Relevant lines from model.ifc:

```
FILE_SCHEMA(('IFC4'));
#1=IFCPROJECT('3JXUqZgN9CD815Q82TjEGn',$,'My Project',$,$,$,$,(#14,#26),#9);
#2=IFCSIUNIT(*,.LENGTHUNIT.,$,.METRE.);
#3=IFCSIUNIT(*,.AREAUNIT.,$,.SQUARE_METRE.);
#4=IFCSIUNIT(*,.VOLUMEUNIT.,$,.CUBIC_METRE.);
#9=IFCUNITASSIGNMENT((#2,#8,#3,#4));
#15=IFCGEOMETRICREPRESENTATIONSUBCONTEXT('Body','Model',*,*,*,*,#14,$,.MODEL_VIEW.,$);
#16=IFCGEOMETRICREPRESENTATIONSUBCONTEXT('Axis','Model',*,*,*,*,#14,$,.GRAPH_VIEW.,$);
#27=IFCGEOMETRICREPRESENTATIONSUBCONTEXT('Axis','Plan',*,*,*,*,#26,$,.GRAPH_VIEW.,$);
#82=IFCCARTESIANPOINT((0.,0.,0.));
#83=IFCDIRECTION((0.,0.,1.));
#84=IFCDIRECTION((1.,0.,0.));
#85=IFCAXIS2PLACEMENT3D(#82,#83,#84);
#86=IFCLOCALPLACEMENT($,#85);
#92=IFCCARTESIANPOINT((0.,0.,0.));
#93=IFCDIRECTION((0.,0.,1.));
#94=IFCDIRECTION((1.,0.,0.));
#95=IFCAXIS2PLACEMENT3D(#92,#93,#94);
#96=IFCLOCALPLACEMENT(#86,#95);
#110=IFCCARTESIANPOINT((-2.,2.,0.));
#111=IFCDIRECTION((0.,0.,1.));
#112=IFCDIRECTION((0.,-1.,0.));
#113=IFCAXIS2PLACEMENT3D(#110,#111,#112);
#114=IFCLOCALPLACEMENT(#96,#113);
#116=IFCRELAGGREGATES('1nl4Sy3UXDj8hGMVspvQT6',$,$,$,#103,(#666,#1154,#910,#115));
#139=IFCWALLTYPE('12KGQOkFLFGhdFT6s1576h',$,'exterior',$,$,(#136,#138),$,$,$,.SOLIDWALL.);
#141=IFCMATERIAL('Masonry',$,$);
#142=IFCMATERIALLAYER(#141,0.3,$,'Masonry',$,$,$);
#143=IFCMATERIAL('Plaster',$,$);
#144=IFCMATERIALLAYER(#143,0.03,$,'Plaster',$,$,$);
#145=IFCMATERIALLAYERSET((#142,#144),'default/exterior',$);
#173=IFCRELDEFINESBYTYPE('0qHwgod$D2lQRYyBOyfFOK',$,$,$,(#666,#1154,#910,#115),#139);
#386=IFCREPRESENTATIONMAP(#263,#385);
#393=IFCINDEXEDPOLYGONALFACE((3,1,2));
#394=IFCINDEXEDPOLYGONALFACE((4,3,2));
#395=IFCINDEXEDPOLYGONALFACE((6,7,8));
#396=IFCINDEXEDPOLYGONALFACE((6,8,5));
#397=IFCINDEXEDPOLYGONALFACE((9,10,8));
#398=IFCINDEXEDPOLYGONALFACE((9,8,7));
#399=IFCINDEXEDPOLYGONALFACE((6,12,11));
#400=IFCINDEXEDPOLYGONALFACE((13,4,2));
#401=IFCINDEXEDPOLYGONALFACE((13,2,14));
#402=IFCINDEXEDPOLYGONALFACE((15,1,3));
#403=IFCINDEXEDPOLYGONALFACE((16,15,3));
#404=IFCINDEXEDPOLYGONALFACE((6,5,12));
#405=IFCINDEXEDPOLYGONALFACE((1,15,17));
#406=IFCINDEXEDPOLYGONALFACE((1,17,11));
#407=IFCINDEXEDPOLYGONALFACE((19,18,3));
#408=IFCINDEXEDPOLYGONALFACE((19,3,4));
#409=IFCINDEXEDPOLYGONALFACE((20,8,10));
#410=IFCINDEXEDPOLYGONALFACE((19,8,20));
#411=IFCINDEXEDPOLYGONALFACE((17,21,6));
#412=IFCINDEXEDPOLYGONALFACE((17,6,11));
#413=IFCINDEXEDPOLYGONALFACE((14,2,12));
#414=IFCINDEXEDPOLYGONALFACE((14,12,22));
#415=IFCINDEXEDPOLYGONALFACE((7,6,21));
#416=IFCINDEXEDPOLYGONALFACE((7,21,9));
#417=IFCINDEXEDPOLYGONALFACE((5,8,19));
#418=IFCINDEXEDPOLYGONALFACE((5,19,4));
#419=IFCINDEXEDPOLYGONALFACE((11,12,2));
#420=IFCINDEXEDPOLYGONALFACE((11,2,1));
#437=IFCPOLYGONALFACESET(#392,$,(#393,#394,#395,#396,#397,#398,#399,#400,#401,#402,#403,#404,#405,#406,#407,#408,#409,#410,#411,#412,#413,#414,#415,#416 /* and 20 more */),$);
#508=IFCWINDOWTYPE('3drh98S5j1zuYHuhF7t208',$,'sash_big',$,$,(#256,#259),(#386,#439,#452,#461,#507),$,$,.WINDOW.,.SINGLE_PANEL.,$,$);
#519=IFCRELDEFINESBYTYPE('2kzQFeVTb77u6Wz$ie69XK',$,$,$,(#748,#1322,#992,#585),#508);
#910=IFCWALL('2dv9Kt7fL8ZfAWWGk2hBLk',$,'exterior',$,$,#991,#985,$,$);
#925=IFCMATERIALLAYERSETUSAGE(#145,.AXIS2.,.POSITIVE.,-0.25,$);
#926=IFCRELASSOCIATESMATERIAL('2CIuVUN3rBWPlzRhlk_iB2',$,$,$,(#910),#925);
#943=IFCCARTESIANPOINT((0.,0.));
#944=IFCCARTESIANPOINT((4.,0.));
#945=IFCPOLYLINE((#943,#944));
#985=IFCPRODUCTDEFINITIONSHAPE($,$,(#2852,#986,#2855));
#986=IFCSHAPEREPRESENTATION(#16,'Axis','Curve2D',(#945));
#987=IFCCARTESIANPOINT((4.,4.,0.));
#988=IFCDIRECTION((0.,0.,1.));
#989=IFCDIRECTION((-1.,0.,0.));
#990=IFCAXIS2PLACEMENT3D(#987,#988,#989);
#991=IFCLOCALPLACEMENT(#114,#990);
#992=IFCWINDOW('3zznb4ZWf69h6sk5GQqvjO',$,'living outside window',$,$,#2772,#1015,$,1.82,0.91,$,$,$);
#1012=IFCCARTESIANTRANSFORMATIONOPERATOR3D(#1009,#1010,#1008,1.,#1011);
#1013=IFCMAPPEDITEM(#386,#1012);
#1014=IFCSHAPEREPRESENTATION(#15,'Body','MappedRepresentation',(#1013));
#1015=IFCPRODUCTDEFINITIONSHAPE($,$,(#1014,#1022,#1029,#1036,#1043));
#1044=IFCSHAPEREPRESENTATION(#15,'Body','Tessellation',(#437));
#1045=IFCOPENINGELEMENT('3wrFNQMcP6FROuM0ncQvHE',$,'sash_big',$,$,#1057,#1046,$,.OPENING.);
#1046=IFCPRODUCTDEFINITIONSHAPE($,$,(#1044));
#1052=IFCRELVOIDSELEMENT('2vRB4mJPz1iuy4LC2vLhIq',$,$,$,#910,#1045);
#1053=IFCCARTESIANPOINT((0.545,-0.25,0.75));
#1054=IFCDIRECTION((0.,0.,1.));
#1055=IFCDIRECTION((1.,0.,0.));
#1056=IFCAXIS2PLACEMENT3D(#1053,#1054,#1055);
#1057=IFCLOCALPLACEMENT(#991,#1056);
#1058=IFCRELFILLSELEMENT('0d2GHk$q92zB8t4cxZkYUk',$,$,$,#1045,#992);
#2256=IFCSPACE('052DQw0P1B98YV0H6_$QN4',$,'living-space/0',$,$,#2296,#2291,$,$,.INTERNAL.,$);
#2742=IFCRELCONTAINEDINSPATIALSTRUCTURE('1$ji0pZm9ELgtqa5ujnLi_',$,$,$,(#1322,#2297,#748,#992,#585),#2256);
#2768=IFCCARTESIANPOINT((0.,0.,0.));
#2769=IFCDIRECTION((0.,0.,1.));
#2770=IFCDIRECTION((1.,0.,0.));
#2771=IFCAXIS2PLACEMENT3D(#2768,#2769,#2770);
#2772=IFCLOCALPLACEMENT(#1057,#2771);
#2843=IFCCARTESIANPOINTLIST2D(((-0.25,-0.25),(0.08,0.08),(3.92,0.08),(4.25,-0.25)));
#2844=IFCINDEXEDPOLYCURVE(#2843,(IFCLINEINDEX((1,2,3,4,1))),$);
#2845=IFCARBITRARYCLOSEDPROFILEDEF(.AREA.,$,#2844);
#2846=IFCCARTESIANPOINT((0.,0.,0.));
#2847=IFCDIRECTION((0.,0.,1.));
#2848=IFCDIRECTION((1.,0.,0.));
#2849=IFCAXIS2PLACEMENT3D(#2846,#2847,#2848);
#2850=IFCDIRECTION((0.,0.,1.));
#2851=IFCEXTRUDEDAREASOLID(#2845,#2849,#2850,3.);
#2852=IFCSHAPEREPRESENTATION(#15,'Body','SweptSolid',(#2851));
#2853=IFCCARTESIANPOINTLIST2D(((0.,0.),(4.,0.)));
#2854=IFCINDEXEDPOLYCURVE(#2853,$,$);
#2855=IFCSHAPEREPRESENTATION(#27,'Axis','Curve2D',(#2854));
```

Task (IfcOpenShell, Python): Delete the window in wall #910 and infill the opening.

```python
import ifcopenshell
import ifcopenshell.api.feature
import ifcopenshell.api.root
import ifcopenshell.geom
import ifcopenshell.util.shape

model = ifcopenshell.open("model.ifc")
settings = ifcopenshell.geom.settings()


def volume(element):
    """Net volume in cubic metres, openings subtracted."""
    shape = ifcopenshell.geom.create_shape(settings, element)
    return ifcopenshell.util.shape.get_volume(shape.geometry)


window = model.by_id(992)
opening = window.FillsVoids[0].RelatingOpeningElement
wall = opening.VoidsElements[0].RelatingBuildingElement
before = volume(wall)

ifcopenshell.api.root.remove_product(model, product=window)
ifcopenshell.api.feature.remove_feature(model, feature=opening)

after = volume(wall)

print(f"wall volume {before:.3f} -> {after:.3f} m3")

model.write("model_edited.ifc")
```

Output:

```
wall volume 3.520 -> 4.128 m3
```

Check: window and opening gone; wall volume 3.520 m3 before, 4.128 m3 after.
